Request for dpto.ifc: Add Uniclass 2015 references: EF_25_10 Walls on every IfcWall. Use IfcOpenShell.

First a look at what the model holds.

```python
import ifcopenshell

model = ifcopenshell.open("dpto.ifc")
print(model.schema)
print("classifications:", [c.Name for c in model.by_type("IfcClassification")])
for ifc_class in ("IfcDoor", "IfcRoof", "IfcStair", "IfcWall", "IfcWindow"):
    print(ifc_class, len(model.by_type(ifc_class)))
```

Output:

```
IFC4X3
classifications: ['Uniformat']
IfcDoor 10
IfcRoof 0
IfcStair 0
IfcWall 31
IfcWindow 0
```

```python
import ifcopenshell
import ifcopenshell.api.classification

model = ifcopenshell.open("dpto.ifc")

system = ifcopenshell.api.classification.add_classification(model, classification="Uniclass 2015")

codes = {
    "IfcWall": ("EF_25_10", "Walls"),
}
for ifc_class, (code, name) in codes.items():
    products = model.by_type(ifc_class)
    ifcopenshell.api.classification.add_reference(
        model, products=products, classification=system, identification=code, name=name
    )
    print(code, len(products))

model.write("dpto_updated.ifc")
```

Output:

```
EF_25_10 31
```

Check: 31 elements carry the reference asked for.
